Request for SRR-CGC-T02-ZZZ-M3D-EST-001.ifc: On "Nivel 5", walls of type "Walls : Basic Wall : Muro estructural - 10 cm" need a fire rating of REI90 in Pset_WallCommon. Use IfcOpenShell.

First a look at what the model holds.

```python
import ifcopenshell
import ifcopenshell.util.element

model = ifcopenshell.open("SRR-CGC-T02-ZZZ-M3D-EST-001.ifc")
print(model.schema)
storey = next(s for s in model.by_type("IfcBuildingStorey") if s.Name == "Nivel 5")
walls = [e for e in ifcopenshell.util.element.get_decomposition(storey) if e.is_a("IfcWall")]
seen = {}
for e in walls:
    element_type = ifcopenshell.util.element.get_type(e)
    key = (element_type.Name if element_type != e and element_type else None, ifcopenshell.util.element.get_pset(e, "Pset_WallCommon", "FireRating"))
    seen[key] = seen.get(key, 0) + 1
for (name, value), count in sorted(seen.items(), key=str):
    print(count, "x", name, "|", value)
```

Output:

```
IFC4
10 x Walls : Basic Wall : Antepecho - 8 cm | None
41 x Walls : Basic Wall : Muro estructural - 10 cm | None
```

```python
import ifcopenshell
import ifcopenshell.api.pset
import ifcopenshell.util.element

model = ifcopenshell.open("SRR-CGC-T02-ZZZ-M3D-EST-001.ifc")

storey = next(s for s in model.by_type("IfcBuildingStorey") if s.Name == "Nivel 5")
walls = [e for e in ifcopenshell.util.element.get_decomposition(storey) if e.is_a("IfcWall")]

count = 0
for e in walls:
    element_type = ifcopenshell.util.element.get_type(e)
    if element_type in (None, e) or element_type.Name != "Walls : Basic Wall : Muro estructural - 10 cm":
        continue
    # add_pset returns the element's existing set when there is one.
    pset = ifcopenshell.api.pset.add_pset(model, product=e, name="Pset_WallCommon")
    ifcopenshell.api.pset.edit_pset(model, pset=pset, properties={"FireRating": "REI90"})
    count += 1

print(count, "walls updated")

model.write("SRR-CGC-T02-ZZZ-M3D-EST-001_updated.ifc")
```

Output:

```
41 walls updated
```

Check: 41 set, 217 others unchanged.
